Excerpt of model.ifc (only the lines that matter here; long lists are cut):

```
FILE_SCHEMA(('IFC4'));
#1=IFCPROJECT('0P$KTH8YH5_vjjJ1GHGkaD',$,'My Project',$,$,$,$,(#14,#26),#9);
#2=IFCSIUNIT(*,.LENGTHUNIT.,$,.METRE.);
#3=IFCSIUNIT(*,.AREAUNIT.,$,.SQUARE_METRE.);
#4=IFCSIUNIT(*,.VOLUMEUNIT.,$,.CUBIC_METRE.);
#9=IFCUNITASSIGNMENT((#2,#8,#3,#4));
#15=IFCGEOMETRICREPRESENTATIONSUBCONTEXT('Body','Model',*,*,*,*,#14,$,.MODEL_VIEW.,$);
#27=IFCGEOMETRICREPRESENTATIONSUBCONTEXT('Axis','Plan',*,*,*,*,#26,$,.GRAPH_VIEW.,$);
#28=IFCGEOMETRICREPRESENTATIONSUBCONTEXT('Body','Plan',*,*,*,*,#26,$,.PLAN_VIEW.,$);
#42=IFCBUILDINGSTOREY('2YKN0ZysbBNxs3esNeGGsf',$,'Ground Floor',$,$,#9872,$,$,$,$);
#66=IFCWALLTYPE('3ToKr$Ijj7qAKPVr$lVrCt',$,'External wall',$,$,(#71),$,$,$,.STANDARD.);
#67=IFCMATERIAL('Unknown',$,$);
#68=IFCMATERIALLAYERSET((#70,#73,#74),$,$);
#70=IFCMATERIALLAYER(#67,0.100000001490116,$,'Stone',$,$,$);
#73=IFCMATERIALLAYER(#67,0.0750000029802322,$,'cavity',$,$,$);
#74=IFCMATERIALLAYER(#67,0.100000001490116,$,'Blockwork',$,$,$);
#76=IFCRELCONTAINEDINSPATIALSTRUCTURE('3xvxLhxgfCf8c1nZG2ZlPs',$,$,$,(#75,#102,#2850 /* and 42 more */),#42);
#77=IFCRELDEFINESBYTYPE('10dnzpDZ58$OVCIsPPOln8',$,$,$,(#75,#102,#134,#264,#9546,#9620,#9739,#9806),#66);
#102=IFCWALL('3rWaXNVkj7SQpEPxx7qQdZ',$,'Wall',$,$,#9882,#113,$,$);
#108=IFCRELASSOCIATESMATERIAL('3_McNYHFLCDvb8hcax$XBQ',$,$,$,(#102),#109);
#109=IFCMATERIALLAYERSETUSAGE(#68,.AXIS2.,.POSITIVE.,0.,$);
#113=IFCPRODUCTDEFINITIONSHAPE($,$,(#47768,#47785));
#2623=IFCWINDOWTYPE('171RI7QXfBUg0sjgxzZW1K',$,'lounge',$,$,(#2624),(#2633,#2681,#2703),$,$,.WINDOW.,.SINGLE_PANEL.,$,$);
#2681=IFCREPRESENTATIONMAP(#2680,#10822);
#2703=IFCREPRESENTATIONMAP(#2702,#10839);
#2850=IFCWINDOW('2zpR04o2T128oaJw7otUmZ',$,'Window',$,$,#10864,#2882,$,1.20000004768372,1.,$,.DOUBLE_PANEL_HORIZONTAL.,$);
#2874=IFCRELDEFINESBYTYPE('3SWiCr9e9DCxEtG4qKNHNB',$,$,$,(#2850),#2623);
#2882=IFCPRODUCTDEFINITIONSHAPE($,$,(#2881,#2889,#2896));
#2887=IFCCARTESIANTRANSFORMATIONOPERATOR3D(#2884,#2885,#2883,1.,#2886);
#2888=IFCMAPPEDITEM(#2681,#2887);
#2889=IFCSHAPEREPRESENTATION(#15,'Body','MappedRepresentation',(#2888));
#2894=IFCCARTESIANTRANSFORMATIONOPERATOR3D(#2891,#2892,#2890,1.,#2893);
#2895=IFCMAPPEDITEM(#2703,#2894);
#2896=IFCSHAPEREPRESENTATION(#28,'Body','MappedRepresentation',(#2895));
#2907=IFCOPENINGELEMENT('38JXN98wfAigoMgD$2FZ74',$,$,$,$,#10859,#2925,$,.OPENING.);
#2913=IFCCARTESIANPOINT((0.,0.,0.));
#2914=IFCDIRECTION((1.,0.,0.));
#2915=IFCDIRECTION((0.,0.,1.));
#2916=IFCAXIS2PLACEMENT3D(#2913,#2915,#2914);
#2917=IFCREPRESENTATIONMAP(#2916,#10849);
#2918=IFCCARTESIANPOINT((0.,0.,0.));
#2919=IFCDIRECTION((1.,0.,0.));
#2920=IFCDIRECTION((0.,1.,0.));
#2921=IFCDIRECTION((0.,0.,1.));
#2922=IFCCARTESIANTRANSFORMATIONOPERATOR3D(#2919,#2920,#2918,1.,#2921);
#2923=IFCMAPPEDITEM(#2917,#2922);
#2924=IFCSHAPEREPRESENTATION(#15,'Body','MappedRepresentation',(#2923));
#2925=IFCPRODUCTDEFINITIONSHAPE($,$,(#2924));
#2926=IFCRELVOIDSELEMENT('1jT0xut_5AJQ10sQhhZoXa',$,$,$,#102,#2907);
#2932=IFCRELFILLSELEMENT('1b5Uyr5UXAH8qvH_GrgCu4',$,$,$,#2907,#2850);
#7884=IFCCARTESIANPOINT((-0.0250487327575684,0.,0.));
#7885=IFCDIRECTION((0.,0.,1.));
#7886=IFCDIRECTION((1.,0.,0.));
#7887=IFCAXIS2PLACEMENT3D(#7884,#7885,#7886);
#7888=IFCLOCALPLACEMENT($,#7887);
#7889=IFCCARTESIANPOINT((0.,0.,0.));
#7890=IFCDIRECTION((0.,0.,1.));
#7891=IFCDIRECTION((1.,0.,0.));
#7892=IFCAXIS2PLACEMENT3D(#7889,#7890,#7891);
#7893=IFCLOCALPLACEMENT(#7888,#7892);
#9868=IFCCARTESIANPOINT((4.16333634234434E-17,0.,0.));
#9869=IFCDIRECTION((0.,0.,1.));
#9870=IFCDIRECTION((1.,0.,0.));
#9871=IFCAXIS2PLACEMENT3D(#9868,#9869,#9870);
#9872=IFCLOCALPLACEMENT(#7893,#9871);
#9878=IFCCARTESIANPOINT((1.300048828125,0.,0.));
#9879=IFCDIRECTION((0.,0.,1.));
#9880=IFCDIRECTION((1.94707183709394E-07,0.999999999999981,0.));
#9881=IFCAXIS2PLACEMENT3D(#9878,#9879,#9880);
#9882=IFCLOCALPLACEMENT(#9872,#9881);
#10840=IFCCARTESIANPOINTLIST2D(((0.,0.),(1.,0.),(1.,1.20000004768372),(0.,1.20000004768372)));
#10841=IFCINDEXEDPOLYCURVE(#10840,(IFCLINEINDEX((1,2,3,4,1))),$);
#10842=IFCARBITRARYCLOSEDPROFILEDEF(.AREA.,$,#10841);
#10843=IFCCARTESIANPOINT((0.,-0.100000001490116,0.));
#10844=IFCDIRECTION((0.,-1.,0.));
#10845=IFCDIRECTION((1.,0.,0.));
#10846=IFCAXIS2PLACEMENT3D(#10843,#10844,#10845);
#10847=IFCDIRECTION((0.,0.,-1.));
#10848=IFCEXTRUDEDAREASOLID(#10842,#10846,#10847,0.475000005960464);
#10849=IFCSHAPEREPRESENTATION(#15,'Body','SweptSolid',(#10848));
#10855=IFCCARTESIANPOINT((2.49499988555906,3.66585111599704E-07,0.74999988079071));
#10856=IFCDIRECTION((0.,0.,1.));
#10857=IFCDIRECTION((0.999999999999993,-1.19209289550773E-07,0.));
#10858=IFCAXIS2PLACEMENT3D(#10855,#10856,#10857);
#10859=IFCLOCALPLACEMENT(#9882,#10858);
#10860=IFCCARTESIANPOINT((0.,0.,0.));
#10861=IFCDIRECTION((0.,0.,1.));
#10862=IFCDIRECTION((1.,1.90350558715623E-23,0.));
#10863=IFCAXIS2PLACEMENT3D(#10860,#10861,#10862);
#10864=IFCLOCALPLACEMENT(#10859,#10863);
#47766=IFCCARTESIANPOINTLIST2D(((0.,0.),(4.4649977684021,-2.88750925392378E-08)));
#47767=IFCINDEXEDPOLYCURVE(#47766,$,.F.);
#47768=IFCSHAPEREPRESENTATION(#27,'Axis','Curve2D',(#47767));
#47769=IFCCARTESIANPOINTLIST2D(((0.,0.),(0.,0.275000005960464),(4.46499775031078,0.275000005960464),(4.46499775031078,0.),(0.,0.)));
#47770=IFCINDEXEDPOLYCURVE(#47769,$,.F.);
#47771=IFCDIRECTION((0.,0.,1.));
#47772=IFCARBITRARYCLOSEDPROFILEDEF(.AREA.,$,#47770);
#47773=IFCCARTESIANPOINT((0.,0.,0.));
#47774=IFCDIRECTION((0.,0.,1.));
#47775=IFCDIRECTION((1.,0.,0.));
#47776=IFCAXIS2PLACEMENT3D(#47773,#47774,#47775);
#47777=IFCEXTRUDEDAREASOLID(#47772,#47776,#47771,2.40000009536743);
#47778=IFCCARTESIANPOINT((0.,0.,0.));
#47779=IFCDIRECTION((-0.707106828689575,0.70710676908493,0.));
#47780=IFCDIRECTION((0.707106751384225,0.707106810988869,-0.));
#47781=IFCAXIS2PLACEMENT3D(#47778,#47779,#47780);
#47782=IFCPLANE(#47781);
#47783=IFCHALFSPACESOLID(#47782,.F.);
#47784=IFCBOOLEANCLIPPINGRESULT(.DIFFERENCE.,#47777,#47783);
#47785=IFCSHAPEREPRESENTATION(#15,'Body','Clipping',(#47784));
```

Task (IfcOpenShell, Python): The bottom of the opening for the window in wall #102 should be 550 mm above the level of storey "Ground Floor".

```python
import numpy as np
import ifcopenshell
import ifcopenshell.api.geometry
import ifcopenshell.geom
import ifcopenshell.util.element
import ifcopenshell.util.placement
import ifcopenshell.util.shape
import ifcopenshell.util.unit

model = ifcopenshell.open("model.ifc")
unit_scale = ifcopenshell.util.unit.calculate_unit_scale(model)

window = model.by_guid("2zpR04o2T128oaJw7otUmZ")
opening = window.FillsVoids[0].RelatingOpeningElement
storey = ifcopenshell.util.element.get_container(window, ifc_class="IfcBuildingStorey")
level = ifcopenshell.util.placement.get_local_placement(storey.ObjectPlacement)[2, 3]

# The opening's origin need not be at the sill, so measure its lowest point.
shape = ifcopenshell.geom.create_shape(ifcopenshell.geom.settings(), opening)
bottom = ifcopenshell.util.shape.get_shape_bottom_elevation(shape, shape.geometry) / unit_scale
dz = level + 0.55 / unit_scale - bottom

shift = np.array([0.0, 0.0, dz])
# The window is placed relative to its opening, so it follows when the opening moves.
matrix = ifcopenshell.util.placement.get_local_placement(opening.ObjectPlacement)
matrix[:3, 3] += shift
ifcopenshell.api.geometry.edit_object_placement(
    model, product=opening, matrix=matrix, is_si=False, should_transform_children=True
)

print(f"moved by {dz * unit_scale:+.3f} m")

model.write("model_rev.ifc")
```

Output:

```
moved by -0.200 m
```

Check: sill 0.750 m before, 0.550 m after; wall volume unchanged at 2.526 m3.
